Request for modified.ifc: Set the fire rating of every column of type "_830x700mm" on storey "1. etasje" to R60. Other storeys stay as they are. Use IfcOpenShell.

First a look at what the model holds.

```python
import ifcopenshell
import ifcopenshell.util.element

model = ifcopenshell.open("modified.ifc")
print(model.schema)
storey = next(s for s in model.by_type("IfcBuildingStorey") if s.Name == "1. etasje")
columns = [e for e in ifcopenshell.util.element.get_decomposition(storey) if e.is_a("IfcColumn")]
seen = {}
for e in columns:
    element_type = ifcopenshell.util.element.get_type(e)
    key = (element_type.Name if element_type != e and element_type else None, ifcopenshell.util.element.get_pset(e, "Pset_ColumnCommon", "FireRating"))
    seen[key] = seen.get(key, 0) + 1
for (name, value), count in sorted(seen.items(), key=str):
    print(count, "x", name, "|", value)
```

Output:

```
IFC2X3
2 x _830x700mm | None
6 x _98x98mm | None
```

```python
import ifcopenshell
import ifcopenshell.api.pset
import ifcopenshell.util.element

model = ifcopenshell.open("modified.ifc")

storey = next(s for s in model.by_type("IfcBuildingStorey") if s.Name == "1. etasje")
columns = [e for e in ifcopenshell.util.element.get_decomposition(storey) if e.is_a("IfcColumn")]

count = 0
for e in columns:
    element_type = ifcopenshell.util.element.get_type(e)
    if element_type in (None, e) or element_type.Name != "_830x700mm":
        continue
    # add_pset returns the element's existing set when there is one.
    pset = ifcopenshell.api.pset.add_pset(model, product=e, name="Pset_ColumnCommon")
    ifcopenshell.api.pset.edit_pset(model, pset=pset, properties={"FireRating": "R60"})
    count += 1

print(count, "columns updated")

model.write("modified_rev.ifc")
```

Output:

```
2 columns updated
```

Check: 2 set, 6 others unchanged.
